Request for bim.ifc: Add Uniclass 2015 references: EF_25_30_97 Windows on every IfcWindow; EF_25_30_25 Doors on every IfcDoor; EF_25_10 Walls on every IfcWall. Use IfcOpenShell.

First a look at what the model holds.

```python
import ifcopenshell

model = ifcopenshell.open("bim.ifc")
print(model.schema)
print("classifications:", [c.Name for c in model.by_type("IfcClassification")])
for ifc_class in ("IfcDoor", "IfcRoof", "IfcStair", "IfcWall", "IfcWindow"):
    print(ifc_class, len(model.by_type(ifc_class)))
```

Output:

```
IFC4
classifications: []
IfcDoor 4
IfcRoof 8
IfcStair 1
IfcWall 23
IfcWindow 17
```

```python
import ifcopenshell
import ifcopenshell.api.classification

model = ifcopenshell.open("bim.ifc")

system = ifcopenshell.api.classification.add_classification(model, classification="Uniclass 2015")

codes = {
    "IfcWindow": ("EF_25_30_97", "Windows"),
    "IfcDoor": ("EF_25_30_25", "Doors"),
    "IfcWall": ("EF_25_10", "Walls"),
}
for ifc_class, (code, name) in codes.items():
    products = model.by_type(ifc_class)
    ifcopenshell.api.classification.add_reference(
        model, products=products, classification=system, identification=code, name=name
    )
    print(code, len(products))

model.write("bim_edited.ifc")
```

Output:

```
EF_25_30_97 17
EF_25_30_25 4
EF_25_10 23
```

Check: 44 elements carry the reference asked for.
